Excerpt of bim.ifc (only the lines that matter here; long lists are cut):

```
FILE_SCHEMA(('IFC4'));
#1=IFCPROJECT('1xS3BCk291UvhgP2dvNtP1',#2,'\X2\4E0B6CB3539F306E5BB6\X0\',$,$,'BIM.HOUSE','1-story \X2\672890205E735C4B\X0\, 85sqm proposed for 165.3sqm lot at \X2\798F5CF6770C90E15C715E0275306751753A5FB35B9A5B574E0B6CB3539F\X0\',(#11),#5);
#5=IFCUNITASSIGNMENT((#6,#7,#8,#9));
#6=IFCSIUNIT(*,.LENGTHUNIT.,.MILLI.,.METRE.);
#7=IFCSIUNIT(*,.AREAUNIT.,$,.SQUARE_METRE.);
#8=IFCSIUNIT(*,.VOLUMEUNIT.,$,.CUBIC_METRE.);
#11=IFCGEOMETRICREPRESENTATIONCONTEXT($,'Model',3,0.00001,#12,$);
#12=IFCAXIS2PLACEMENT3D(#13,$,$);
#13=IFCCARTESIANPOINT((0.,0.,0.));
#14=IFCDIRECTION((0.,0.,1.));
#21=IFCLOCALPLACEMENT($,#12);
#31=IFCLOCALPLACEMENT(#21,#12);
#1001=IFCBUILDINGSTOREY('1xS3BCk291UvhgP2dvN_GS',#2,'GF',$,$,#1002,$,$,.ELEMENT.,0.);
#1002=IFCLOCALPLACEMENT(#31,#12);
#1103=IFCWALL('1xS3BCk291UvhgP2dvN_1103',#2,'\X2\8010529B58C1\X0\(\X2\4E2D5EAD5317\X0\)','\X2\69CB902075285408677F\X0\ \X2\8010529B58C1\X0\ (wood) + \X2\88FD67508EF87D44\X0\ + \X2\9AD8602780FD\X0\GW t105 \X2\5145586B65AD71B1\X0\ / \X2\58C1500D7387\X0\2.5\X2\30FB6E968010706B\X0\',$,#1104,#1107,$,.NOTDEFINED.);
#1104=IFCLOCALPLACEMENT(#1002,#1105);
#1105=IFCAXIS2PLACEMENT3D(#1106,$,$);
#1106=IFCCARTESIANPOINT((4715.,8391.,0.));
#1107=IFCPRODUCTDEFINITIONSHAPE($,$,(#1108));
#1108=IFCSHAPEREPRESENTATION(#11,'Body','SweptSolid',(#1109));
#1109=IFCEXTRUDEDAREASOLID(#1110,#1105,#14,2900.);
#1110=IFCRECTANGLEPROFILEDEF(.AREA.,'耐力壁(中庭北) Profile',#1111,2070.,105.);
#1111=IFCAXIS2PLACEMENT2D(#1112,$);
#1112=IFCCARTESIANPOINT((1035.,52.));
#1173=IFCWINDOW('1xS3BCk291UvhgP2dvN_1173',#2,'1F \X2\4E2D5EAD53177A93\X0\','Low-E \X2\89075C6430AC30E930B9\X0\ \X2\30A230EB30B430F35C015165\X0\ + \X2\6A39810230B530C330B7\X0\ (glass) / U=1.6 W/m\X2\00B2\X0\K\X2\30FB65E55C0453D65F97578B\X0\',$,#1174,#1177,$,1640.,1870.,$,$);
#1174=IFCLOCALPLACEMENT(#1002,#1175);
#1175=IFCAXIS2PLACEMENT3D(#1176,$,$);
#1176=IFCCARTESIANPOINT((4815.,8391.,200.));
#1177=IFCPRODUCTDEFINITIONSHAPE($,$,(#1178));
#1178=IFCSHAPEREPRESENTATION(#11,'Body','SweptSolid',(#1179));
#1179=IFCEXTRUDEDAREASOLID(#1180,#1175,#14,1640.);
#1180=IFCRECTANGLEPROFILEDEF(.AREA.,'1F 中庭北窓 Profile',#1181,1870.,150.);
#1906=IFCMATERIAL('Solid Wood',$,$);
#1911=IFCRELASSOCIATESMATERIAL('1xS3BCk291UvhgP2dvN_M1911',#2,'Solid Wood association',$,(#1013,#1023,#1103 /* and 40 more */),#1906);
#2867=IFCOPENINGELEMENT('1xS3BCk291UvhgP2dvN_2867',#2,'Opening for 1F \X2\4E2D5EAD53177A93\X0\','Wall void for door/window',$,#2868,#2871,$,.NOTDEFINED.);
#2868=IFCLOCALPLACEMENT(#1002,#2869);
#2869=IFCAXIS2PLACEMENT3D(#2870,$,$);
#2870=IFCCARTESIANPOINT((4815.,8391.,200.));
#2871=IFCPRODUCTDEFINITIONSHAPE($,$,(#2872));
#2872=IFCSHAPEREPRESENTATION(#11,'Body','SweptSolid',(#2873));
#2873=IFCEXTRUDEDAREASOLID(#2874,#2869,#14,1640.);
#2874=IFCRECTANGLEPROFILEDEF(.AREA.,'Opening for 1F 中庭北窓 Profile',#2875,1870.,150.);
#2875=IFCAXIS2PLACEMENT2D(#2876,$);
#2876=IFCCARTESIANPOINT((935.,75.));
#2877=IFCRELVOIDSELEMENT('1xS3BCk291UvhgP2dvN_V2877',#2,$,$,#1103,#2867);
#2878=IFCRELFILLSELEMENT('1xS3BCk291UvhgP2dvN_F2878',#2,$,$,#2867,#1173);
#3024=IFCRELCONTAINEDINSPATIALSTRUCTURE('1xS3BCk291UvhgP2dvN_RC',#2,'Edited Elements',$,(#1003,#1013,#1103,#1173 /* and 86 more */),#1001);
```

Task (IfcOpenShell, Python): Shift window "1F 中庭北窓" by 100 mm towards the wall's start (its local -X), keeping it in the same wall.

```python
import ifcopenshell
import ifcopenshell.api.geometry
import ifcopenshell.util.placement

model = ifcopenshell.open("bim.ifc")

window = model.by_guid("1xS3BCk291UvhgP2dvN_1173")
opening = window.FillsVoids[0].RelatingOpeningElement
wall = opening.VoidsElements[0].RelatingBuildingElement

wall_matrix = ifcopenshell.util.placement.get_local_placement(wall.ObjectPlacement)
shift = wall_matrix[:3, 0] * -100.0
before = ifcopenshell.util.placement.get_local_placement(window.ObjectPlacement)[:3, 3].copy()

# The window is not placed relative to its opening, so move both.
for product in (opening, window):
    matrix = ifcopenshell.util.placement.get_local_placement(product.ObjectPlacement)
    matrix[:3, 3] += shift
    ifcopenshell.api.geometry.edit_object_placement(model, product=product, matrix=matrix, is_si=False)

after = ifcopenshell.util.placement.get_local_placement(window.ObjectPlacement)[:3, 3]
print("window moved by", (after - before).round(3) + 0.0)

model.write("bim_updated.ifc")
```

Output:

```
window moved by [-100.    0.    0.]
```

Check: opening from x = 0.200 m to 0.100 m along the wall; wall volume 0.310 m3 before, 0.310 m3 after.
